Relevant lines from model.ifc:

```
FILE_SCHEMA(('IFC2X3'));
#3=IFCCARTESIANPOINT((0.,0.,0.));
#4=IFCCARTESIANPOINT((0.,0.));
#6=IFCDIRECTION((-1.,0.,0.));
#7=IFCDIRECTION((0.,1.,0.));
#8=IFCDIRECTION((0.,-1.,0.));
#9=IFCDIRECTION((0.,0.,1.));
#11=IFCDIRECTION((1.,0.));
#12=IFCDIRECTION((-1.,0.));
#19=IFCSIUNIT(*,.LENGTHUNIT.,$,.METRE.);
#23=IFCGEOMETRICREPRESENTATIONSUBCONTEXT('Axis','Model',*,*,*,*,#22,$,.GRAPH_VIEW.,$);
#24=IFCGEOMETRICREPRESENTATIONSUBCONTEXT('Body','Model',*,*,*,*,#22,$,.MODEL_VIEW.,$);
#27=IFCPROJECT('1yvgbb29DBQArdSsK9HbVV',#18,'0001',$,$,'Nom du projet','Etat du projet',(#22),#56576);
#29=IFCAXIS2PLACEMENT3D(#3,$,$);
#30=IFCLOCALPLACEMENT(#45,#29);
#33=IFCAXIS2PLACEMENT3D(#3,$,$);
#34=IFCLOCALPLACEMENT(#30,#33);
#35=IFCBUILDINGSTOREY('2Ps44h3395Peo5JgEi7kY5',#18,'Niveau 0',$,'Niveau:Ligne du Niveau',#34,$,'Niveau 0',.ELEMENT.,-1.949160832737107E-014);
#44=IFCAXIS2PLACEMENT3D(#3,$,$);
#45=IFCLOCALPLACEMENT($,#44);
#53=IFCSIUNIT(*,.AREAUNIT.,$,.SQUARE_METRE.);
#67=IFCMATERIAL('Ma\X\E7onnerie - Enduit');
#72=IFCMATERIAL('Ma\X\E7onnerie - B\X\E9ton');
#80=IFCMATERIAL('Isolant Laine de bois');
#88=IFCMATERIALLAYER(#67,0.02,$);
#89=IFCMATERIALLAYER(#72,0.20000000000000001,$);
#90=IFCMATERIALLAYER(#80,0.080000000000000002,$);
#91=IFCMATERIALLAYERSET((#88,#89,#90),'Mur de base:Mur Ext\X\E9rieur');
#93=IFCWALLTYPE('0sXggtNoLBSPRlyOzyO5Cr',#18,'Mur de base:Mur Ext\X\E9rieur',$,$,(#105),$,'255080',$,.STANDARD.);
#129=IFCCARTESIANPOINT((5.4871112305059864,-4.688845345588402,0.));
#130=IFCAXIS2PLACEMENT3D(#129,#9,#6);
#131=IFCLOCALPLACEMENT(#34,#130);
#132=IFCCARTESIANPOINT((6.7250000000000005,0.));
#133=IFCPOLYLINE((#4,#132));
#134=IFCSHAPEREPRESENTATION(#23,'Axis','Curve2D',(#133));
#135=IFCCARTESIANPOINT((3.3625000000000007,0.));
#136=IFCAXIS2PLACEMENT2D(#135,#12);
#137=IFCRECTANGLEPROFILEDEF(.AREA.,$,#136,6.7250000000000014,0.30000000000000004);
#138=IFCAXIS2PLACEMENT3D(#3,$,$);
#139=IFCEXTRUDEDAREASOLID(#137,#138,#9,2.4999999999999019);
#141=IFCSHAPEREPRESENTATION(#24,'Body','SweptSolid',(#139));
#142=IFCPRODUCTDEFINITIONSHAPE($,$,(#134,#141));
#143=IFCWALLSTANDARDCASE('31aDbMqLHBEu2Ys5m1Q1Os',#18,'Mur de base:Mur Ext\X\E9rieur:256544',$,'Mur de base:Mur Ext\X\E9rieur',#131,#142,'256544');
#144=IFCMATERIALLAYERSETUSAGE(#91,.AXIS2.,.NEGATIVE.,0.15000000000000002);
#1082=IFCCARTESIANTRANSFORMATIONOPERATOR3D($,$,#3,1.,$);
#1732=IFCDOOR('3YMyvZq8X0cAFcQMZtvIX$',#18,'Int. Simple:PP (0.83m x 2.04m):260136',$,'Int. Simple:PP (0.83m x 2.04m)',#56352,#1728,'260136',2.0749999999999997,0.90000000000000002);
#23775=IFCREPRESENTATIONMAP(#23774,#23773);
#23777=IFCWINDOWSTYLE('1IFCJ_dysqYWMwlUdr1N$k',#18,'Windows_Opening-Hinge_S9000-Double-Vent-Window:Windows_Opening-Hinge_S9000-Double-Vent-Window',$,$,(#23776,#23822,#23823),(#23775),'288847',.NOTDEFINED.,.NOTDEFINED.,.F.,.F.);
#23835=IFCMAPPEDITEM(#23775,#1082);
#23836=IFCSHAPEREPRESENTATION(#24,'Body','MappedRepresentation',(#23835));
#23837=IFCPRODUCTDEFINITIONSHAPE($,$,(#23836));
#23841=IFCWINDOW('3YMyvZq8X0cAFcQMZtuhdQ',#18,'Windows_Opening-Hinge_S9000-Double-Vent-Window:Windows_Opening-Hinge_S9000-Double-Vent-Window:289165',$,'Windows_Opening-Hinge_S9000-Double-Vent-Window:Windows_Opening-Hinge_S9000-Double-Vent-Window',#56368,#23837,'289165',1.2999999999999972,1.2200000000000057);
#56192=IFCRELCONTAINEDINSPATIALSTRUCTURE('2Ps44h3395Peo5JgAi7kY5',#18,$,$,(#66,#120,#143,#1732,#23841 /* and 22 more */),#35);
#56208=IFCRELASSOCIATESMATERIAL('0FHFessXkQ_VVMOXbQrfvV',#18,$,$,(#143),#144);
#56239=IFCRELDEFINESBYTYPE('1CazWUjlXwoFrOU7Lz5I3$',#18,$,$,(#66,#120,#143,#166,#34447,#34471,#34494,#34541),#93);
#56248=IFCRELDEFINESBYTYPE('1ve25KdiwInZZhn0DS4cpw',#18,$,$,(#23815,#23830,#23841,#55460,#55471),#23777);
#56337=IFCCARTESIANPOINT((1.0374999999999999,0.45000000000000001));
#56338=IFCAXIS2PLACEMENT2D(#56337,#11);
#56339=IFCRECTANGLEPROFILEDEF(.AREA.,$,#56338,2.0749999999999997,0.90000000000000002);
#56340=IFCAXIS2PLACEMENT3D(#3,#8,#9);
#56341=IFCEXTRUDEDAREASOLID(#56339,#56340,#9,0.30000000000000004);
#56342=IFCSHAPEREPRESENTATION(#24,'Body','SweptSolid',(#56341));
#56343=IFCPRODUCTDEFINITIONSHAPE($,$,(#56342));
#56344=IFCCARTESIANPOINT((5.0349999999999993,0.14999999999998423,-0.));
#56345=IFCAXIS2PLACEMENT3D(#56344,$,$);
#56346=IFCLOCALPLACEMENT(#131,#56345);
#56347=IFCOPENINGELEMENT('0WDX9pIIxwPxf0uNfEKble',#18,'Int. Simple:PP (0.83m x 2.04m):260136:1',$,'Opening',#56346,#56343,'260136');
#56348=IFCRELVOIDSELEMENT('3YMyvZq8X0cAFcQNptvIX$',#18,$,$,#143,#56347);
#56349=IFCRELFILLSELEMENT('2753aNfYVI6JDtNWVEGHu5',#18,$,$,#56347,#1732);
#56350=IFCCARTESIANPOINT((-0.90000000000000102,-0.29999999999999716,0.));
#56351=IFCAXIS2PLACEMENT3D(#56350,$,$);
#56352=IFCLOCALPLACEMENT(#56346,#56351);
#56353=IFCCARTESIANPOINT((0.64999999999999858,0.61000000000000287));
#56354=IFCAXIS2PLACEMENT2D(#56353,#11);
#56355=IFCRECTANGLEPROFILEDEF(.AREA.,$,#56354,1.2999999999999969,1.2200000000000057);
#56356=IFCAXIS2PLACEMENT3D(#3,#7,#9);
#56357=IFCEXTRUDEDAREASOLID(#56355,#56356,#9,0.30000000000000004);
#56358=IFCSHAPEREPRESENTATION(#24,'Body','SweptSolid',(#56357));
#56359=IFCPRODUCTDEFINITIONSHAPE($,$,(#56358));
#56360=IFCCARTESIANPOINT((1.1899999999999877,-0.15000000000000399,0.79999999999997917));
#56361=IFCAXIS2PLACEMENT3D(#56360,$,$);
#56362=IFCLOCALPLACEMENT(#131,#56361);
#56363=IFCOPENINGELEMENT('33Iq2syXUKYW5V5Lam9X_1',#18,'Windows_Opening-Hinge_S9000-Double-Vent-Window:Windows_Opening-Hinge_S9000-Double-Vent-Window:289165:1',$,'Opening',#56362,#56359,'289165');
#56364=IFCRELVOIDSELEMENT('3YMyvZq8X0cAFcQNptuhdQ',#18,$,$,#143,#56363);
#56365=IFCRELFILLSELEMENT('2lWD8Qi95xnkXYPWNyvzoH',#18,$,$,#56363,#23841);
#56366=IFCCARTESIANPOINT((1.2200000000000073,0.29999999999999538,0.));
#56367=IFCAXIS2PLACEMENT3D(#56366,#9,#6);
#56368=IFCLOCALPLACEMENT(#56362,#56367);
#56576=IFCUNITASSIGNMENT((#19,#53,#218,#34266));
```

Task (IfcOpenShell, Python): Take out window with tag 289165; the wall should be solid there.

```python
import ifcopenshell
import ifcopenshell.api.feature
import ifcopenshell.api.root
import ifcopenshell.geom
import ifcopenshell.util.shape

model = ifcopenshell.open("model.ifc")
settings = ifcopenshell.geom.settings()


def volume(element):
    """Net volume in cubic metres, openings subtracted."""
    shape = ifcopenshell.geom.create_shape(settings, element)
    return ifcopenshell.util.shape.get_volume(shape.geometry)


window = model.by_id(23841)
opening = window.FillsVoids[0].RelatingOpeningElement
wall = opening.VoidsElements[0].RelatingBuildingElement
before = volume(wall)

ifcopenshell.api.root.remove_product(model, product=window)
ifcopenshell.api.feature.remove_feature(model, feature=opening)

after = volume(wall)

print(f"wall volume {before:.3f} -> {after:.3f} m3")

model.write("model_rev.ifc")
```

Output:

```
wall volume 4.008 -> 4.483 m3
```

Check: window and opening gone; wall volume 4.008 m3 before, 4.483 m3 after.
